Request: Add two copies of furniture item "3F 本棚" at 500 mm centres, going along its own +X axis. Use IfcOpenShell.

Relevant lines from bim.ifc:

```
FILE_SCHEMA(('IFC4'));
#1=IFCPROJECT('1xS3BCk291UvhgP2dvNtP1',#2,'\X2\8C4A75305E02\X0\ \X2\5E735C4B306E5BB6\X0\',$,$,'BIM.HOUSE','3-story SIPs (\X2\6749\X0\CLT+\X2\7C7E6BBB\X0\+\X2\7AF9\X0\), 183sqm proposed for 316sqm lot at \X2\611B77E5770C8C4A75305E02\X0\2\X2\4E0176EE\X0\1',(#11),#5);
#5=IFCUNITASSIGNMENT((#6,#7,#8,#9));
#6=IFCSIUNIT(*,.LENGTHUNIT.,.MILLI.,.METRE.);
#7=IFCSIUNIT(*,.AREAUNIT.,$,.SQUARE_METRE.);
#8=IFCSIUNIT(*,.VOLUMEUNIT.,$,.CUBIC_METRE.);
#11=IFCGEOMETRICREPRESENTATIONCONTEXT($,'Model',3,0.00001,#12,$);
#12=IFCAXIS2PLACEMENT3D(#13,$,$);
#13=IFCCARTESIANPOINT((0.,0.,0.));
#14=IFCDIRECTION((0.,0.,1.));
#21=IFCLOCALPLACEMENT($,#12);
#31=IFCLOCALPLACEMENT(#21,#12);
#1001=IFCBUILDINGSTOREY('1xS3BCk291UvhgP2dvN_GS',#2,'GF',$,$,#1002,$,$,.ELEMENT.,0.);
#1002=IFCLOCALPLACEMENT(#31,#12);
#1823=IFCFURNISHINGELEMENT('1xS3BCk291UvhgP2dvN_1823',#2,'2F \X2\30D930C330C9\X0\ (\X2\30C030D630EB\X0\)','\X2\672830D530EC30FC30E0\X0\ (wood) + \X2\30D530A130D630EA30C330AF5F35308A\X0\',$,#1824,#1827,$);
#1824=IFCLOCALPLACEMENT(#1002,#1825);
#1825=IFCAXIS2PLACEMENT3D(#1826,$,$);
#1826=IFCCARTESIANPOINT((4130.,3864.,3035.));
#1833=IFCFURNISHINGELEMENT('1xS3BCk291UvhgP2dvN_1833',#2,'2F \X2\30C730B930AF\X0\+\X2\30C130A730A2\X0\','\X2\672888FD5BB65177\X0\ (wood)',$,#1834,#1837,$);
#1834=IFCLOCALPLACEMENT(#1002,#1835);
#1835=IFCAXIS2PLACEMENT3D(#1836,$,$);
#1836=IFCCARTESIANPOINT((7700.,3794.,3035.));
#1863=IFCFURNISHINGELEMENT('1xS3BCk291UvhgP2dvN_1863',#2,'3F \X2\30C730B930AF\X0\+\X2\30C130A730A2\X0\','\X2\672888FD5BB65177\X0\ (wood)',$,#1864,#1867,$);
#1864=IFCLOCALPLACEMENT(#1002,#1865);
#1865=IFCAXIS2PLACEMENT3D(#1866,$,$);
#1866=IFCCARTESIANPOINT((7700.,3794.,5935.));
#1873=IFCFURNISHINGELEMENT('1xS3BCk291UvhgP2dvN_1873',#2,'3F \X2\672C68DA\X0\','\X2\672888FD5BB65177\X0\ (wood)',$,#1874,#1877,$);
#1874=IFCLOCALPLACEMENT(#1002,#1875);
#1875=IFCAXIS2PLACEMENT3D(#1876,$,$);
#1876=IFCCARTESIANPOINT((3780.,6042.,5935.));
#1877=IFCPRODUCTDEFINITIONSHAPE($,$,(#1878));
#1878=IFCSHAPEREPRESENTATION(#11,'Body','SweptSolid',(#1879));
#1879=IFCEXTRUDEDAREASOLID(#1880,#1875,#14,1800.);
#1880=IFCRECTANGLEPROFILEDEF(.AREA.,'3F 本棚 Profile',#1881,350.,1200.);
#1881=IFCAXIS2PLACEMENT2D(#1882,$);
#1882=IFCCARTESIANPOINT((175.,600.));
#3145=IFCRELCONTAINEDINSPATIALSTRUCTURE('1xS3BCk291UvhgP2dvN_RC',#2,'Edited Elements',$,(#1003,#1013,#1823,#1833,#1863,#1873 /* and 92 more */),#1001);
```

```python
import ifcopenshell
import ifcopenshell.api.geometry
import ifcopenshell.api.root
import ifcopenshell.util.element
import ifcopenshell.util.placement

model = ifcopenshell.open("bim.ifc")


def reuse_history(source, copy):
    """copy_class also copies each property set's owner history, people and application; keep the originals."""
    for rel in copy.IsDefinedBy:
        if rel.is_a("IfcRelDefinesByProperties") and (history := rel.RelatingPropertyDefinition.OwnerHistory):
            rel.RelatingPropertyDefinition.OwnerHistory = source.OwnerHistory
            ifcopenshell.util.element.remove_deep2(model, history)


source = model.by_id(1873)
base = ifcopenshell.util.placement.get_local_placement(source.ObjectPlacement)
step = base[:3, 0] * 500.0

for i in range(1, 3):
    copy = ifcopenshell.api.root.copy_class(model, product=source)
    copy.Representation = ifcopenshell.util.element.copy_deep(
        model, source.Representation, exclude=["IfcGeometricRepresentationContext", "IfcRepresentationMap"]
    )
    reuse_history(source, copy)
    matrix = base.copy()
    matrix[:3, 3] += i * step
    print("added at", matrix[:3, 3].round(3) + 0.0)
    ifcopenshell.api.geometry.edit_object_placement(model, product=copy, matrix=matrix, is_si=False)

model.write("bim_v2.ifc")
```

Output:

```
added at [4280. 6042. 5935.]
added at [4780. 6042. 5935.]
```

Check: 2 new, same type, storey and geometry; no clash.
